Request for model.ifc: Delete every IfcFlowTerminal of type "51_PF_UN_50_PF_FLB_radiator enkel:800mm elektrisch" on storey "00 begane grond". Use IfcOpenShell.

First a look at what the model holds.

```python
import ifcopenshell
import ifcopenshell.util.element

model = ifcopenshell.open("model.ifc")
print(model.schema)
storey = next(s for s in model.by_type("IfcBuildingStorey") if s.Name == "00 begane grond")
terminals = [e for e in ifcopenshell.util.element.get_decomposition(storey) if e.is_a("IfcFlowTerminal")]
seen = {}
for e in terminals:
    element_type = ifcopenshell.util.element.get_type(e)
    name = element_type.Name if element_type not in (None, e) else None
    seen[name] = seen.get(name, 0) + 1
for name, count in sorted(seen.items(), key=str):
    print(count, "x", name)
```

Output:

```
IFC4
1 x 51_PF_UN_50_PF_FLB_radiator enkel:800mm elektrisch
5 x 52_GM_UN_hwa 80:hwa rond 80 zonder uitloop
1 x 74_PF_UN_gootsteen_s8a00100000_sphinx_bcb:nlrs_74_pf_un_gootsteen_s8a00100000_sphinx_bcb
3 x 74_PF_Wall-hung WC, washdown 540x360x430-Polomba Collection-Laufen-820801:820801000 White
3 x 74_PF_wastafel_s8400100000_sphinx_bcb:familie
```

```python
import ifcopenshell
import ifcopenshell.api.root
import ifcopenshell.util.element

model = ifcopenshell.open("model.ifc")

storey = next(s for s in model.by_type("IfcBuildingStorey") if s.Name == "00 begane grond")
terminals = [e for e in ifcopenshell.util.element.get_decomposition(storey) if e.is_a("IfcFlowTerminal")]
targets = [e for e in terminals if (t := ifcopenshell.util.element.get_type(e)) not in (None, e) and t.Name == "51_PF_UN_50_PF_FLB_radiator enkel:800mm elektrisch"]

for e in targets:
    ifcopenshell.api.root.remove_product(model, product=e)
print(len(targets), "removed")

model.write("model_edited.ifc")
```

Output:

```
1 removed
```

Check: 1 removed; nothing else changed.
